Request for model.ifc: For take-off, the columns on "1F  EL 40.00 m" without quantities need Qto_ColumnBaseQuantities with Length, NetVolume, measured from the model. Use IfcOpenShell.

First a look at what the model holds.

```python
import ifcopenshell
import ifcopenshell.util.element
import ifcopenshell.util.unit

model = ifcopenshell.open("model.ifc")
print(model.schema)
for unit_type in ("LENGTHUNIT", "AREAUNIT", "VOLUMEUNIT"):
    print(unit_type, ifcopenshell.util.unit.calculate_unit_scale(model, unit_type))
storey = next(s for s in model.by_type("IfcBuildingStorey") if s.Name == "1F  EL 40.00 m")
columns = [e for e in ifcopenshell.util.element.get_decomposition(storey) if e.is_a("IfcColumn")]
for e in sorted(columns, key=lambda e: e.id()):
    print(e.id(), e.is_a(), e.Name, list(ifcopenshell.util.element.get_psets(e, qtos_only=True)), sep=" | ")
```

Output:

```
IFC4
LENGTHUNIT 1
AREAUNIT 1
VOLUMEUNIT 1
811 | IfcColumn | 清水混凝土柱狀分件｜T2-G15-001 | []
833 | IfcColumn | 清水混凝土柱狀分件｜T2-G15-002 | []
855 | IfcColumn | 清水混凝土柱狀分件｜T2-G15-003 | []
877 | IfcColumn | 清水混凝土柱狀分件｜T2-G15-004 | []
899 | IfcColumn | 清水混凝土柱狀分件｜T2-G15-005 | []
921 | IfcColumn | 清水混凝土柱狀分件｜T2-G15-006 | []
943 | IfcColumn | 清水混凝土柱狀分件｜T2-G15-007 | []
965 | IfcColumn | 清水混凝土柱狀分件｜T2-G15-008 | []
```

```python
import ifcopenshell
import ifcopenshell.api.pset
import ifcopenshell.geom
import ifcopenshell.util.element
import ifcopenshell.util.shape
import ifcopenshell.util.unit

model = ifcopenshell.open("model.ifc")
unit_scale = ifcopenshell.util.unit.calculate_unit_scale(model)
volume_scale = ifcopenshell.util.unit.calculate_unit_scale(model, "VOLUMEUNIT")
settings = ifcopenshell.geom.settings()

storey = next(s for s in model.by_type("IfcBuildingStorey") if s.Name == "1F  EL 40.00 m")
columns = [e for e in ifcopenshell.util.element.get_decomposition(storey) if e.is_a("IfcColumn")]

for e in sorted(columns, key=lambda e: e.id()):
    if ifcopenshell.util.element.get_psets(e, qtos_only=True, should_inherit=False):
        continue
    # Geometry comes back in metres, in the element's own axes.
    shape = ifcopenshell.geom.create_shape(settings, e)
    values = {
        "Length": ifcopenshell.util.shape.get_z(shape.geometry) / unit_scale,
        "NetVolume": ifcopenshell.util.shape.get_volume(shape.geometry) / volume_scale,
    }
    qto = ifcopenshell.api.pset.add_qto(model, product=e, name="Qto_ColumnBaseQuantities")
    ifcopenshell.api.pset.edit_qto(model, qto=qto, properties=values)
    print(e.id(), {k: round(v, 3) for k, v in values.items()})

model.write("model_edited.ifc")
```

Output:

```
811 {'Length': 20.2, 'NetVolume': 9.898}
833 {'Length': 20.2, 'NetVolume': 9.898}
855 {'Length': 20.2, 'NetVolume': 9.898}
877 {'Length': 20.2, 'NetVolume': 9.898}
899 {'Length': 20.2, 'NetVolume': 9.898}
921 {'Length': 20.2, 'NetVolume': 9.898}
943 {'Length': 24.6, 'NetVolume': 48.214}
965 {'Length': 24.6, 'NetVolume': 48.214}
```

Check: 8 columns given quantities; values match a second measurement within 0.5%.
